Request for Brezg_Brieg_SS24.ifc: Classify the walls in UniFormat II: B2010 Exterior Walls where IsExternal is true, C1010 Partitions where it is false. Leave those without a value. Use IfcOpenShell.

First a look at what the model holds.

```python
import ifcopenshell
import ifcopenshell.util.element

model = ifcopenshell.open("Brezg_Brieg_SS24.ifc")
print(model.schema)
print("classifications:", [c.Name for c in model.by_type("IfcClassification")])
values = [ifcopenshell.util.element.get_pset(e, "Pset_WallCommon", "IsExternal") for e in model.by_type("IfcWall")]
for value in (True, False, None):
    print("IsExternal", value, values.count(value))
```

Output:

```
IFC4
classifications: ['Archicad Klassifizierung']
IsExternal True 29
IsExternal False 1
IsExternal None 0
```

```python
import ifcopenshell
import ifcopenshell.api.classification
import ifcopenshell.util.element

model = ifcopenshell.open("Brezg_Brieg_SS24.ifc")

system = ifcopenshell.api.classification.add_classification(model, classification="UniFormat II")

walls = model.by_type("IfcWall")
external = {e: ifcopenshell.util.element.get_pset(e, "Pset_WallCommon", "IsExternal") for e in walls}
for flag, code, name in ((True, "B2010", "Exterior Walls"), (False, "C1010", "Partitions")):
    products = [e for e in walls if external[e] is flag]
    ifcopenshell.api.classification.add_reference(
        model, products=products, classification=system, identification=code, name=name
    )
    print(code, len(products))

model.write("Brezg_Brieg_SS24_edited.ifc")
```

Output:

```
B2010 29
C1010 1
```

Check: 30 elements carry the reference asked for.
